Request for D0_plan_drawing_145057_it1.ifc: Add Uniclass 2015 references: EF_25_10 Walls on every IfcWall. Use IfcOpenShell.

First a look at what the model holds.

```python
import ifcopenshell

model = ifcopenshell.open("D0_plan_drawing_145057_it1.ifc")
print(model.schema)
print("classifications:", [c.Name for c in model.by_type("IfcClassification")])
for ifc_class in ("IfcDoor", "IfcRoof", "IfcStair", "IfcWall", "IfcWindow"):
    print(ifc_class, len(model.by_type(ifc_class)))
```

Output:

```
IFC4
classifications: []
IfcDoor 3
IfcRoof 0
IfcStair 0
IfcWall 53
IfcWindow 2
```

```python
import ifcopenshell
import ifcopenshell.api.classification

model = ifcopenshell.open("D0_plan_drawing_145057_it1.ifc")

system = ifcopenshell.api.classification.add_classification(model, classification="Uniclass 2015")

codes = {
    "IfcWall": ("EF_25_10", "Walls"),
}
for ifc_class, (code, name) in codes.items():
    products = model.by_type(ifc_class)
    ifcopenshell.api.classification.add_reference(
        model, products=products, classification=system, identification=code, name=name
    )
    print(code, len(products))

model.write("D0_plan_drawing_145057_it1_edited.ifc")
```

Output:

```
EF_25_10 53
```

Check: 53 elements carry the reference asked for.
